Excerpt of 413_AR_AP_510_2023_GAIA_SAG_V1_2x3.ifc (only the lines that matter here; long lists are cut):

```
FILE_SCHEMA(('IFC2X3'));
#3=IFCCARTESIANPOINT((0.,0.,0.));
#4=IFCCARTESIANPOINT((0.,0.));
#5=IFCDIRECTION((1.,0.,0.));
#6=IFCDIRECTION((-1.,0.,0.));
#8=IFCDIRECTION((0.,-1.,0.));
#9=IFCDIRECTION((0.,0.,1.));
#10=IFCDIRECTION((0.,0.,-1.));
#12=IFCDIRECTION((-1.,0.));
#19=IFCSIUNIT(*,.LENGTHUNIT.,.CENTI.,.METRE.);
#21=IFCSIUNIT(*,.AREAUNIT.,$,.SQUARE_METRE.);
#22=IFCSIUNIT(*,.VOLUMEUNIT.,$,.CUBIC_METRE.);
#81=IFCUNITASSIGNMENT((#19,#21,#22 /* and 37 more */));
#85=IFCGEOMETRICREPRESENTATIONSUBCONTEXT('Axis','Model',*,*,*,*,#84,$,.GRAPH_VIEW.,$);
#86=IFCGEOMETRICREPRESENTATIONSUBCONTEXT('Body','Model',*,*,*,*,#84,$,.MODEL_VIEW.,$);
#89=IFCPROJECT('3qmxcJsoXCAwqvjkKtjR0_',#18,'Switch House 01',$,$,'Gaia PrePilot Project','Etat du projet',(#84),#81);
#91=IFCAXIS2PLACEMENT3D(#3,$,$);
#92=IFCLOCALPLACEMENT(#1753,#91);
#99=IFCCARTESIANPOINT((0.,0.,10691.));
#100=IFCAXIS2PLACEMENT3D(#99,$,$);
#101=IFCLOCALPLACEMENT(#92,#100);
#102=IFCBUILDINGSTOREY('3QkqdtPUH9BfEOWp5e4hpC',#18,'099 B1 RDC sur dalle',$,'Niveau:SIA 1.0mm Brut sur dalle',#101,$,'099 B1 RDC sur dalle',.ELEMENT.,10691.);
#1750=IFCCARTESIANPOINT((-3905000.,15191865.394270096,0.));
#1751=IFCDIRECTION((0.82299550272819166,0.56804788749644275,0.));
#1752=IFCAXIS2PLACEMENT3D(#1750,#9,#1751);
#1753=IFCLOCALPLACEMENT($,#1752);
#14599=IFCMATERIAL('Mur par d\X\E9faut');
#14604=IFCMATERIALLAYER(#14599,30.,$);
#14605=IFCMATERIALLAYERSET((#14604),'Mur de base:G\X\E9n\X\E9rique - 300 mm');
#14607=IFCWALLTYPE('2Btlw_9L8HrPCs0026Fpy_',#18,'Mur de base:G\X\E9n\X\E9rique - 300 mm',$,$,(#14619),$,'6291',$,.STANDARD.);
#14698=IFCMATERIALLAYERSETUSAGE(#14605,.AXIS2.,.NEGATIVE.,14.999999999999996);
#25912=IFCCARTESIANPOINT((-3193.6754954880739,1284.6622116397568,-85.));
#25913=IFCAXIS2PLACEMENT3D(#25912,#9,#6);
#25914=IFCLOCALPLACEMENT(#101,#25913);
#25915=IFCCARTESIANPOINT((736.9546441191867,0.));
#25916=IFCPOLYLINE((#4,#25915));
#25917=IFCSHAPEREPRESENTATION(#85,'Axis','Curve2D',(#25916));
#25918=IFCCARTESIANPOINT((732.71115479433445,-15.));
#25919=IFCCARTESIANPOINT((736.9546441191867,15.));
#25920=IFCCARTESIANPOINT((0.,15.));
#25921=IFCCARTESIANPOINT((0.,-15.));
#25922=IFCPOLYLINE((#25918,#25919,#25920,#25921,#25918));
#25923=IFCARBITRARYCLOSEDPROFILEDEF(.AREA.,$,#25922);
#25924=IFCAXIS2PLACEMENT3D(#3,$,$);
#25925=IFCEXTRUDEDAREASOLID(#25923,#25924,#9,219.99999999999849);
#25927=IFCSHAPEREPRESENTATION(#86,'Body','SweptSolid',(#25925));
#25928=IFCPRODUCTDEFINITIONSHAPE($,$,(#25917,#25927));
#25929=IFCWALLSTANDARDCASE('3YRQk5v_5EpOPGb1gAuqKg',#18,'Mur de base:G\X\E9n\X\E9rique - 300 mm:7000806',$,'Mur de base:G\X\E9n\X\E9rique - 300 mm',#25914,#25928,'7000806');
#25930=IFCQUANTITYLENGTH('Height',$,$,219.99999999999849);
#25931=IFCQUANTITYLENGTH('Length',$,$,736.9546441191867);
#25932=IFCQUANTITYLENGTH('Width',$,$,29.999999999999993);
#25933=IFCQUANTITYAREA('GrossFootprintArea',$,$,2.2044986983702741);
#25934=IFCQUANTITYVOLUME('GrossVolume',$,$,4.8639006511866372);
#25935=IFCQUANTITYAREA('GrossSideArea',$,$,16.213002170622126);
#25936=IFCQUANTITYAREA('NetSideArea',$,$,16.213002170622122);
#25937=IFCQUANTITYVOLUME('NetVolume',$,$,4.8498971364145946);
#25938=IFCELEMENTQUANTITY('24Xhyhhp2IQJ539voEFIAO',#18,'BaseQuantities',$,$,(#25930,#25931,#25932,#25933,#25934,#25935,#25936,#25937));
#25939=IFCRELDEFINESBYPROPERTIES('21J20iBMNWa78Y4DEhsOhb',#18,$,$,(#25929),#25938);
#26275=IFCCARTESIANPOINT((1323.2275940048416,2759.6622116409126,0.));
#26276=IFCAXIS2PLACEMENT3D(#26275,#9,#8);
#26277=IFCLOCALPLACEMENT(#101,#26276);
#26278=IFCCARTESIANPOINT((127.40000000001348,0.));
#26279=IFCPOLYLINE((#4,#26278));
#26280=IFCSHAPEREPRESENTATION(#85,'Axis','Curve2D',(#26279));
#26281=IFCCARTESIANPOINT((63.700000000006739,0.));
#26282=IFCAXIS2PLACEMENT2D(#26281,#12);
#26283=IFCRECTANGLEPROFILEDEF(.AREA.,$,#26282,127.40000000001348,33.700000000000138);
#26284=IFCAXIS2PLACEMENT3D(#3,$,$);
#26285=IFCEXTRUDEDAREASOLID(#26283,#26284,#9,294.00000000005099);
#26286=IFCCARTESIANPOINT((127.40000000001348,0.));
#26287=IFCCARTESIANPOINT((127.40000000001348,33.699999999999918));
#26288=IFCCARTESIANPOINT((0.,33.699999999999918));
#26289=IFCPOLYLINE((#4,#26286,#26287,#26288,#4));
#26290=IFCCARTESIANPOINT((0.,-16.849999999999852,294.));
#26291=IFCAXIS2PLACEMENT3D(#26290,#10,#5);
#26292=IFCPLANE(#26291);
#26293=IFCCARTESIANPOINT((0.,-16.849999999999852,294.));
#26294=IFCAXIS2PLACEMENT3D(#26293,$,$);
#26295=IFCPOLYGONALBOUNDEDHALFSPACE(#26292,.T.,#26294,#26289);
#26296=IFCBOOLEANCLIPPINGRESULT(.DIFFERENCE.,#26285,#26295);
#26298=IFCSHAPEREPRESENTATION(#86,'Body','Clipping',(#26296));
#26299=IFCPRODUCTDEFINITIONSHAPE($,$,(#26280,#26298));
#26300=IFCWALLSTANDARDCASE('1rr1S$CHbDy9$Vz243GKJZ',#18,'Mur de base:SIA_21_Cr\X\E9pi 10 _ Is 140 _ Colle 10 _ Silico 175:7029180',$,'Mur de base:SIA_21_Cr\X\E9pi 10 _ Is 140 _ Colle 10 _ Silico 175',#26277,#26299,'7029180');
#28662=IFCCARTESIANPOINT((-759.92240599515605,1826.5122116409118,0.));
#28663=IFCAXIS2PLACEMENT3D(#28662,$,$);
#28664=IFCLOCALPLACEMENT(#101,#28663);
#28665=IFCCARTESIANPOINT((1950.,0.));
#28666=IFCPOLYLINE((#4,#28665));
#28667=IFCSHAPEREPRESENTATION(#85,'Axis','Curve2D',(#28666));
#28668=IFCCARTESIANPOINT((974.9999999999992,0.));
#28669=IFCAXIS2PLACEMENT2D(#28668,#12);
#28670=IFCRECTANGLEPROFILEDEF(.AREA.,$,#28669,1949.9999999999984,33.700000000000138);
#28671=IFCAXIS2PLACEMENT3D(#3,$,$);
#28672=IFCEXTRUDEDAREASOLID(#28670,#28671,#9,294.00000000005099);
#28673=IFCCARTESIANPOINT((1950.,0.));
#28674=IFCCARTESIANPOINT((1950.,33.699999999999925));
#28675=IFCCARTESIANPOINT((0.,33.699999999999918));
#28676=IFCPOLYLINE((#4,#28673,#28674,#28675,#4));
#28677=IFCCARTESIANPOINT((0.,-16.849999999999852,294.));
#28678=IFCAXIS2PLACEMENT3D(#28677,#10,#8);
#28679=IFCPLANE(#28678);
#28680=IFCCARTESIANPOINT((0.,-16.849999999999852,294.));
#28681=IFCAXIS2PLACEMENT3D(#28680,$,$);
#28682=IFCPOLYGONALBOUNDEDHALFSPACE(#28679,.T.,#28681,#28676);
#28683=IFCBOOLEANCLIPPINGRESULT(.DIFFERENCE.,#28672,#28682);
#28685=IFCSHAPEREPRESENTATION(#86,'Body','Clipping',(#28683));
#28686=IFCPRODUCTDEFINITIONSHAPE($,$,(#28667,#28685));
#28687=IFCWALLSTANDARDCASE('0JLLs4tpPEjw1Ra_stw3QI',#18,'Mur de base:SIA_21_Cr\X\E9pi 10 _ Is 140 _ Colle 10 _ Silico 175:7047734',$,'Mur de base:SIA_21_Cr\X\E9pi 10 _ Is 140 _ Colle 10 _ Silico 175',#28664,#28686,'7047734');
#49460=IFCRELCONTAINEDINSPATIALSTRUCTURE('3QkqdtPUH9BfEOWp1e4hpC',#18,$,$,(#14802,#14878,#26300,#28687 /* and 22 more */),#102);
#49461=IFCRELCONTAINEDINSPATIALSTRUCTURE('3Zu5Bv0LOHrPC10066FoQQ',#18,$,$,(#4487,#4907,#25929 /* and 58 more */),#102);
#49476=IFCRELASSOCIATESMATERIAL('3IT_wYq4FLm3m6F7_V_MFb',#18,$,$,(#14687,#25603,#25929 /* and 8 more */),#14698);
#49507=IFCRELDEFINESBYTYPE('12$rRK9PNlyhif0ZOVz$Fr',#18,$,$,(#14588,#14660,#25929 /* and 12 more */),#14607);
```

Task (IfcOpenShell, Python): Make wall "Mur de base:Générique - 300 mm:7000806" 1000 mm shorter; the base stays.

```python
import ifcopenshell
import ifcopenshell.api.pset
import ifcopenshell.geom
import ifcopenshell.util.element
import ifcopenshell.util.representation
import ifcopenshell.util.shape
import ifcopenshell.util.unit

model = ifcopenshell.open("413_AR_AP_510_2023_GAIA_SAG_V1_2x3.ifc")
unit_scale = ifcopenshell.util.unit.calculate_unit_scale(model)
area_scale = ifcopenshell.util.unit.calculate_unit_scale(model, "AREAUNIT")
volume_scale = ifcopenshell.util.unit.calculate_unit_scale(model, "VOLUMEUNIT")
settings = ifcopenshell.geom.settings()


def volume(element):
    """Net volume in cubic metres, openings subtracted."""
    shape = ifcopenshell.geom.create_shape(settings, element)
    return ifcopenshell.util.shape.get_volume(shape.geometry)


wall = model.by_guid("3YRQk5v_5EpOPGb1gAuqKg")
before = volume(wall)

body = ifcopenshell.util.representation.get_representation(wall, "Model", "Body")
solid = body.Items[0]
old_height = solid.Depth
solid.Depth -= 1 / unit_scale
after = volume(wall)
thickness = 0.3  # wall thickness in metres

# Update the stored height, areas and volumes.
qto = model.by_id(ifcopenshell.util.element.get_pset(wall, "BaseQuantities", should_inherit=False)["id"])
ifcopenshell.api.pset.edit_qto(model, qto=qto, properties={
    "Height": solid.Depth,
    "GrossVolume": ifcopenshell.util.element.get_pset(wall, "BaseQuantities", "GrossVolume") * solid.Depth / old_height,
    "GrossSideArea": ifcopenshell.util.element.get_pset(wall, "BaseQuantities", "GrossSideArea") * solid.Depth / old_height,
    "NetSideArea": after / thickness / area_scale,
    "NetVolume": after / volume_scale,
})

print(f"height {old_height:g} -> {solid.Depth:g}, volume {before:.3f} -> {after:.3f} m3")

model.write("413_AR_AP_510_2023_GAIA_SAG_V1_2x3-out.ifc")
```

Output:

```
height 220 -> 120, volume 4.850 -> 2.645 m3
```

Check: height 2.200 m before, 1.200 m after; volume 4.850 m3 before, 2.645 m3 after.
